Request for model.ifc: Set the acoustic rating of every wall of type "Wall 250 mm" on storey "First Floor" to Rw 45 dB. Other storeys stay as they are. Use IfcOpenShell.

First a look at what the model holds.

```python
import ifcopenshell
import ifcopenshell.util.element

model = ifcopenshell.open("model.ifc")
print(model.schema)
storey = next(s for s in model.by_type("IfcBuildingStorey") if s.Name == "First Floor")
walls = [e for e in ifcopenshell.util.element.get_decomposition(storey) if e.is_a("IfcWall")]
seen = {}
for e in walls:
    element_type = ifcopenshell.util.element.get_type(e)
    key = (element_type.Name if element_type != e and element_type else None, ifcopenshell.util.element.get_pset(e, "Pset_WallCommon", "AcousticRating"))
    seen[key] = seen.get(key, 0) + 1
for (name, value), count in sorted(seen.items(), key=str):
    print(count, "x", name, "|", value)
```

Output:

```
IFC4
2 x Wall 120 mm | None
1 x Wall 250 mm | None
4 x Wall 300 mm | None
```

```python
import ifcopenshell
import ifcopenshell.api.pset
import ifcopenshell.util.element

model = ifcopenshell.open("model.ifc")

storey = next(s for s in model.by_type("IfcBuildingStorey") if s.Name == "First Floor")
walls = [e for e in ifcopenshell.util.element.get_decomposition(storey) if e.is_a("IfcWall")]

count = 0
for e in walls:
    element_type = ifcopenshell.util.element.get_type(e)
    if element_type in (None, e) or element_type.Name != "Wall 250 mm":
        continue
    # add_pset returns the element's existing set when there is one.
    pset = ifcopenshell.api.pset.add_pset(model, product=e, name="Pset_WallCommon")
    ifcopenshell.api.pset.edit_pset(model, pset=pset, properties={"AcousticRating": "Rw 45 dB"})
    count += 1

print(count, "walls updated")

model.write("model_edited.ifc")
```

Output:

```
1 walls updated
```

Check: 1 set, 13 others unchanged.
